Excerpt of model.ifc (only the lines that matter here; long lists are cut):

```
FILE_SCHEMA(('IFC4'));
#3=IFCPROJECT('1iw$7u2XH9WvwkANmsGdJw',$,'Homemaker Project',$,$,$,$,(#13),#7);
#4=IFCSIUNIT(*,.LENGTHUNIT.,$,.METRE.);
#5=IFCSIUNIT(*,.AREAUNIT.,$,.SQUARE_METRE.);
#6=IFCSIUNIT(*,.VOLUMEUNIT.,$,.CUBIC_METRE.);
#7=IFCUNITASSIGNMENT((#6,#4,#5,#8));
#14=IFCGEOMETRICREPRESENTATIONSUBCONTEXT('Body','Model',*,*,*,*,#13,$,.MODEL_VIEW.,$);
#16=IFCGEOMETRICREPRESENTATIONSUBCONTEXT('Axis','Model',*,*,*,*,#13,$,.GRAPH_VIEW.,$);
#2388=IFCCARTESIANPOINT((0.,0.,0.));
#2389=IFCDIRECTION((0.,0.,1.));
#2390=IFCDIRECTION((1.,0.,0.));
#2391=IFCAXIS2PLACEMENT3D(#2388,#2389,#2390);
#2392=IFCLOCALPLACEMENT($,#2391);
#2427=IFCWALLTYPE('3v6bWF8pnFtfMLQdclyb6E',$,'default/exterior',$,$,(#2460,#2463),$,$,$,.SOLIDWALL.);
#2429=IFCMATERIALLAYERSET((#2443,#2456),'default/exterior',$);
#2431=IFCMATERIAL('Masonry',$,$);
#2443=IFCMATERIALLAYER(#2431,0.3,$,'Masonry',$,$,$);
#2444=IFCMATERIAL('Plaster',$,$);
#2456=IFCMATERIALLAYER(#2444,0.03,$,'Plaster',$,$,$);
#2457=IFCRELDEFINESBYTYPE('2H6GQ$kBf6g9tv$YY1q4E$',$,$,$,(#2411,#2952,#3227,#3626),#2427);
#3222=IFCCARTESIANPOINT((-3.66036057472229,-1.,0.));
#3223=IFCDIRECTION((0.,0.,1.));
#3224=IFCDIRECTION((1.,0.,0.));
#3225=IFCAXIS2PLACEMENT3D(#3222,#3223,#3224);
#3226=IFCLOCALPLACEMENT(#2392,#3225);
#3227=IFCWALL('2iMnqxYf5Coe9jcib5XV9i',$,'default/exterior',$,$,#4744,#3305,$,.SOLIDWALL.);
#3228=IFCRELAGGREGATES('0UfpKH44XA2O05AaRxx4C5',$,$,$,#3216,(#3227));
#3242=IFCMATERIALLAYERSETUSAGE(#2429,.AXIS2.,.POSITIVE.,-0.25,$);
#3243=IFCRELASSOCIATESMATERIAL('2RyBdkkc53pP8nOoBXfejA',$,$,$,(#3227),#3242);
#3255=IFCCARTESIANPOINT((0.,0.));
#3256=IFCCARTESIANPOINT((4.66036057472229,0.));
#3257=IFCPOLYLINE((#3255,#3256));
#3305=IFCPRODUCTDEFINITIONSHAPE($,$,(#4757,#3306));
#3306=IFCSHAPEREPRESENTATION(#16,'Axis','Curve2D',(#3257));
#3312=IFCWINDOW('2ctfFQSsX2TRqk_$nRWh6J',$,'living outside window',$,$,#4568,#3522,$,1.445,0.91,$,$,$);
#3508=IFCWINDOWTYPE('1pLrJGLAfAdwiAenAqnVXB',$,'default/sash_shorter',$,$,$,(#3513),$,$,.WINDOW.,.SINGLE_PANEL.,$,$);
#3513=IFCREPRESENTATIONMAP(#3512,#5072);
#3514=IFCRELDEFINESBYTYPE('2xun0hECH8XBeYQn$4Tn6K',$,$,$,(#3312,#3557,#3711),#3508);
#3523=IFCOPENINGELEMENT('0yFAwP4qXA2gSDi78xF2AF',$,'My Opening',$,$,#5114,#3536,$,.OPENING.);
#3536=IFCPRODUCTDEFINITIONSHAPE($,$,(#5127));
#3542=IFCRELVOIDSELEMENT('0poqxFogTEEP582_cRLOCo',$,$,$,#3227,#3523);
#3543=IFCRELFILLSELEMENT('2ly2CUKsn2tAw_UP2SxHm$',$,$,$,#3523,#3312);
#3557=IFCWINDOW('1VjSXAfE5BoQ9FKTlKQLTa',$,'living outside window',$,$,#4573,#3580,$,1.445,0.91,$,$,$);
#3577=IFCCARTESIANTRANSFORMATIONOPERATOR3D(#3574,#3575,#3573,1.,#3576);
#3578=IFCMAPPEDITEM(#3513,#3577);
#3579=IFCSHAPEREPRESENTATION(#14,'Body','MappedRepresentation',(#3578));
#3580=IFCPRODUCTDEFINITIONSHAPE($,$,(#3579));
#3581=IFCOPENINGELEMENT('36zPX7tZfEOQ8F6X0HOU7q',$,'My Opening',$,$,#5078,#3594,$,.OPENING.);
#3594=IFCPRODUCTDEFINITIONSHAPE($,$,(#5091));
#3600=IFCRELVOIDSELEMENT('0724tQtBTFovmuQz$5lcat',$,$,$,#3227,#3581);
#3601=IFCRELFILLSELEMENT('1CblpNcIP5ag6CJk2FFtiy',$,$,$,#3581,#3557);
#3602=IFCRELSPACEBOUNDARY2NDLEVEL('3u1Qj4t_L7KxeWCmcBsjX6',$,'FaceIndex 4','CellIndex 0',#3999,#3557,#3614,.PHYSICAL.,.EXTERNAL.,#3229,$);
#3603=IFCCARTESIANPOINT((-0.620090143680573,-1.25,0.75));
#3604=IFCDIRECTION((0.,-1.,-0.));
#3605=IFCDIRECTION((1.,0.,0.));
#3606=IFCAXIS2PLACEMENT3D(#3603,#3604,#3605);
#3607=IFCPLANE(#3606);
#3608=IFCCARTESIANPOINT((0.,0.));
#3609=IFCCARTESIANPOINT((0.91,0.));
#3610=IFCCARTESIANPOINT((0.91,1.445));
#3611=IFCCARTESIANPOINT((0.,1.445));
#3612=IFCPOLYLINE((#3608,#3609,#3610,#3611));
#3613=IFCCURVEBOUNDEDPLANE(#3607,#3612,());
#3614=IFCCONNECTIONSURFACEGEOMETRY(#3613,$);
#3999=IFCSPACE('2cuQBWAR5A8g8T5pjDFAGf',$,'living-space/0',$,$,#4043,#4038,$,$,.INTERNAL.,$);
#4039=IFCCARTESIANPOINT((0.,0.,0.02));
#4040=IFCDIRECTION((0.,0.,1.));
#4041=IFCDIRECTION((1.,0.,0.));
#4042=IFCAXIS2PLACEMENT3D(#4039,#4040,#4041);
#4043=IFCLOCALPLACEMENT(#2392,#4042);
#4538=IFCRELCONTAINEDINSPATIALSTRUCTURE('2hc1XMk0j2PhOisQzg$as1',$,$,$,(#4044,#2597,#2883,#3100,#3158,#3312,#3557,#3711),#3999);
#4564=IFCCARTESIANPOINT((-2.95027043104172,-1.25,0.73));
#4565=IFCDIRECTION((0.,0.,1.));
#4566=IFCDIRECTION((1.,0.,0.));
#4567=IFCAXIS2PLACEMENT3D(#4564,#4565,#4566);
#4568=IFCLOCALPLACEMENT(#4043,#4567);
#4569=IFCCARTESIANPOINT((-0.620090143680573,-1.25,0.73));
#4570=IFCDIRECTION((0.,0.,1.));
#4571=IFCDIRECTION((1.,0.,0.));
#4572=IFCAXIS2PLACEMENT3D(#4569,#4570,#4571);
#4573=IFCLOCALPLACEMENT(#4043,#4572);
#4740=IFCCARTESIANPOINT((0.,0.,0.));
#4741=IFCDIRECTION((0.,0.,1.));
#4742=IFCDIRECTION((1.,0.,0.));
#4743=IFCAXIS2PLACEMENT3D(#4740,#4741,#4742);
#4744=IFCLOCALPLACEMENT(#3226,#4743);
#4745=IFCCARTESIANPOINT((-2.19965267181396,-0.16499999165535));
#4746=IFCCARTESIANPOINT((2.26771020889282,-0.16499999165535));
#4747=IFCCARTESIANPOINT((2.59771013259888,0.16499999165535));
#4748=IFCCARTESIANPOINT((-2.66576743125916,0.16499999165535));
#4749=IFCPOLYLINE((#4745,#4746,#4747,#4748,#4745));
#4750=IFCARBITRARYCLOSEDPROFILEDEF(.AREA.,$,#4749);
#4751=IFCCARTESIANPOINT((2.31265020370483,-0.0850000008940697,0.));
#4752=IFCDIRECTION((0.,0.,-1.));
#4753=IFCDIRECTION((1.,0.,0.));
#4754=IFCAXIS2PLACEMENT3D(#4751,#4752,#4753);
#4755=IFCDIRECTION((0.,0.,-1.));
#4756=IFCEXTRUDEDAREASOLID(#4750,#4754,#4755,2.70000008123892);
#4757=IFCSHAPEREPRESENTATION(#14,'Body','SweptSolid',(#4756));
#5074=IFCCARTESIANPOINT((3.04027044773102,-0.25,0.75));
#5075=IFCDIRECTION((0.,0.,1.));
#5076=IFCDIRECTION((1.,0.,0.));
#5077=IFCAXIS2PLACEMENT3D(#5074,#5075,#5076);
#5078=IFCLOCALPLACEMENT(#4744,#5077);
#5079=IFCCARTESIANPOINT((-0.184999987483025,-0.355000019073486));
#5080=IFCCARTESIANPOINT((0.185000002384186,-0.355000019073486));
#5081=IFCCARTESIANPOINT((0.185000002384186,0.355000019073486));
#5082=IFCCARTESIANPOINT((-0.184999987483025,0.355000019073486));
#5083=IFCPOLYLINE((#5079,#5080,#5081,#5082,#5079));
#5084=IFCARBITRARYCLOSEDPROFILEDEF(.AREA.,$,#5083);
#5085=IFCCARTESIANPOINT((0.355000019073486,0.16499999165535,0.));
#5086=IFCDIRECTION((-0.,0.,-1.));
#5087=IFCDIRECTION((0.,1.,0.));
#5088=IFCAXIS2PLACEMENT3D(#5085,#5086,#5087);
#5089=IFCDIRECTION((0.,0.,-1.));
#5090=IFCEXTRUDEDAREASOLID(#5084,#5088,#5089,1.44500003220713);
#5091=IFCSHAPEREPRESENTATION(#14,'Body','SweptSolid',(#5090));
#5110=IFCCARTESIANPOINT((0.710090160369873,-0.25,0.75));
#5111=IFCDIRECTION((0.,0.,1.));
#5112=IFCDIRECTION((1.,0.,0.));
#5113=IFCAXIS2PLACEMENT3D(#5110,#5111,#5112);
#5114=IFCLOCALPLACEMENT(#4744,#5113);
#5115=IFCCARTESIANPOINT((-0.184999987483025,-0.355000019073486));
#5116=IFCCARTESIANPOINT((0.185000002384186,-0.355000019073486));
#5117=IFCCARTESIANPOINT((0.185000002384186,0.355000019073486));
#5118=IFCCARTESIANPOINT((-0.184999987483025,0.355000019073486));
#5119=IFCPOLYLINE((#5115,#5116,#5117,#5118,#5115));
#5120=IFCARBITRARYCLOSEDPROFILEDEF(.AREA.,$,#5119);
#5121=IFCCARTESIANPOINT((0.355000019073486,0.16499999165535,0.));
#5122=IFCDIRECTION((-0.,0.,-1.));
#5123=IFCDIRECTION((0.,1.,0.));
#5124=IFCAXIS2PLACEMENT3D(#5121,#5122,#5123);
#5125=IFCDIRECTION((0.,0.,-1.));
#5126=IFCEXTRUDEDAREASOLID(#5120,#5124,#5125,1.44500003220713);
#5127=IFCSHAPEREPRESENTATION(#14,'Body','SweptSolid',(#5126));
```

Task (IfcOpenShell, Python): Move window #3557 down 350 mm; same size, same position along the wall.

```python
import numpy as np
import ifcopenshell
import ifcopenshell.api.geometry
import ifcopenshell.util.placement
import ifcopenshell.util.unit

model = ifcopenshell.open("model.ifc")
unit_scale = ifcopenshell.util.unit.calculate_unit_scale(model)

window = model.by_guid("1VjSXAfE5BoQ9FKTlKQLTa")
opening = window.FillsVoids[0].RelatingOpeningElement
dz = -0.35

shift = np.array([0.0, 0.0, dz])
# The window is not placed relative to its opening, so move both.
for product in (opening, window):
    matrix = ifcopenshell.util.placement.get_local_placement(product.ObjectPlacement)
    matrix[:3, 3] += shift
    ifcopenshell.api.geometry.edit_object_placement(model, product=product, matrix=matrix, is_si=False)

# Space boundary surfaces are stored in each space's coordinates; move them too.
for rel in window.ProvidesBoundaries:
    if not rel.ConnectionGeometry:
        continue
    surface = rel.ConnectionGeometry.SurfaceOnRelatingElement.BasisSurface
    space_matrix = ifcopenshell.util.placement.get_local_placement(rel.RelatingSpace.ObjectPlacement)
    point = np.array(surface.Position.Location.Coordinates) + space_matrix[:3, :3].T @ shift
    surface.Position = model.createIfcAxis2Placement3D(
        model.createIfcCartesianPoint(point.tolist()), surface.Position.Axis, surface.Position.RefDirection
    )

print(f"moved by {dz * unit_scale:+.3f} m")

model.write("model_updated.ifc")
```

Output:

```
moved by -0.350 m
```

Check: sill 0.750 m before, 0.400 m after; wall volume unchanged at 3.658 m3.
